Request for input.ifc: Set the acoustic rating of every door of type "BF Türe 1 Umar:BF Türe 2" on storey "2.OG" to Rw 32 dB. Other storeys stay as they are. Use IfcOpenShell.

First a look at what the model holds.

```python
import ifcopenshell
import ifcopenshell.util.element

model = ifcopenshell.open("input.ifc")
print(model.schema)
storey = next(s for s in model.by_type("IfcBuildingStorey") if s.Name == "2.OG")
doors = [e for e in ifcopenshell.util.element.get_decomposition(storey) if e.is_a("IfcDoor")]
seen = {}
for e in doors:
    element_type = ifcopenshell.util.element.get_type(e)
    key = (element_type.Name if element_type != e and element_type else None, ifcopenshell.util.element.get_pset(e, "Pset_DoorCommon", "AcousticRating"))
    seen[key] = seen.get(key, 0) + 1
for (name, value), count in sorted(seen.items(), key=str):
    print(count, "x", name, "|", value)
```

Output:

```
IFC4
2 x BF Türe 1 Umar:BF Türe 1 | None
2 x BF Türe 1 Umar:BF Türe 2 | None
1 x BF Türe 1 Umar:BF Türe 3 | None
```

```python
import ifcopenshell
import ifcopenshell.api.pset
import ifcopenshell.util.element

model = ifcopenshell.open("input.ifc")

storey = next(s for s in model.by_type("IfcBuildingStorey") if s.Name == "2.OG")
doors = [e for e in ifcopenshell.util.element.get_decomposition(storey) if e.is_a("IfcDoor")]

count = 0
for e in doors:
    element_type = ifcopenshell.util.element.get_type(e)
    if element_type in (None, e) or element_type.Name != "BF Türe 1 Umar:BF Türe 2":
        continue
    # add_pset returns the element's existing set when there is one.
    pset = ifcopenshell.api.pset.add_pset(model, product=e, name="Pset_DoorCommon")
    ifcopenshell.api.pset.edit_pset(model, pset=pset, properties={"AcousticRating": "Rw 32 dB"})
    count += 1

print(count, "doors updated")

model.write("input_updated.ifc")
```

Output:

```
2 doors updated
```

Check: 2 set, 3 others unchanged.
